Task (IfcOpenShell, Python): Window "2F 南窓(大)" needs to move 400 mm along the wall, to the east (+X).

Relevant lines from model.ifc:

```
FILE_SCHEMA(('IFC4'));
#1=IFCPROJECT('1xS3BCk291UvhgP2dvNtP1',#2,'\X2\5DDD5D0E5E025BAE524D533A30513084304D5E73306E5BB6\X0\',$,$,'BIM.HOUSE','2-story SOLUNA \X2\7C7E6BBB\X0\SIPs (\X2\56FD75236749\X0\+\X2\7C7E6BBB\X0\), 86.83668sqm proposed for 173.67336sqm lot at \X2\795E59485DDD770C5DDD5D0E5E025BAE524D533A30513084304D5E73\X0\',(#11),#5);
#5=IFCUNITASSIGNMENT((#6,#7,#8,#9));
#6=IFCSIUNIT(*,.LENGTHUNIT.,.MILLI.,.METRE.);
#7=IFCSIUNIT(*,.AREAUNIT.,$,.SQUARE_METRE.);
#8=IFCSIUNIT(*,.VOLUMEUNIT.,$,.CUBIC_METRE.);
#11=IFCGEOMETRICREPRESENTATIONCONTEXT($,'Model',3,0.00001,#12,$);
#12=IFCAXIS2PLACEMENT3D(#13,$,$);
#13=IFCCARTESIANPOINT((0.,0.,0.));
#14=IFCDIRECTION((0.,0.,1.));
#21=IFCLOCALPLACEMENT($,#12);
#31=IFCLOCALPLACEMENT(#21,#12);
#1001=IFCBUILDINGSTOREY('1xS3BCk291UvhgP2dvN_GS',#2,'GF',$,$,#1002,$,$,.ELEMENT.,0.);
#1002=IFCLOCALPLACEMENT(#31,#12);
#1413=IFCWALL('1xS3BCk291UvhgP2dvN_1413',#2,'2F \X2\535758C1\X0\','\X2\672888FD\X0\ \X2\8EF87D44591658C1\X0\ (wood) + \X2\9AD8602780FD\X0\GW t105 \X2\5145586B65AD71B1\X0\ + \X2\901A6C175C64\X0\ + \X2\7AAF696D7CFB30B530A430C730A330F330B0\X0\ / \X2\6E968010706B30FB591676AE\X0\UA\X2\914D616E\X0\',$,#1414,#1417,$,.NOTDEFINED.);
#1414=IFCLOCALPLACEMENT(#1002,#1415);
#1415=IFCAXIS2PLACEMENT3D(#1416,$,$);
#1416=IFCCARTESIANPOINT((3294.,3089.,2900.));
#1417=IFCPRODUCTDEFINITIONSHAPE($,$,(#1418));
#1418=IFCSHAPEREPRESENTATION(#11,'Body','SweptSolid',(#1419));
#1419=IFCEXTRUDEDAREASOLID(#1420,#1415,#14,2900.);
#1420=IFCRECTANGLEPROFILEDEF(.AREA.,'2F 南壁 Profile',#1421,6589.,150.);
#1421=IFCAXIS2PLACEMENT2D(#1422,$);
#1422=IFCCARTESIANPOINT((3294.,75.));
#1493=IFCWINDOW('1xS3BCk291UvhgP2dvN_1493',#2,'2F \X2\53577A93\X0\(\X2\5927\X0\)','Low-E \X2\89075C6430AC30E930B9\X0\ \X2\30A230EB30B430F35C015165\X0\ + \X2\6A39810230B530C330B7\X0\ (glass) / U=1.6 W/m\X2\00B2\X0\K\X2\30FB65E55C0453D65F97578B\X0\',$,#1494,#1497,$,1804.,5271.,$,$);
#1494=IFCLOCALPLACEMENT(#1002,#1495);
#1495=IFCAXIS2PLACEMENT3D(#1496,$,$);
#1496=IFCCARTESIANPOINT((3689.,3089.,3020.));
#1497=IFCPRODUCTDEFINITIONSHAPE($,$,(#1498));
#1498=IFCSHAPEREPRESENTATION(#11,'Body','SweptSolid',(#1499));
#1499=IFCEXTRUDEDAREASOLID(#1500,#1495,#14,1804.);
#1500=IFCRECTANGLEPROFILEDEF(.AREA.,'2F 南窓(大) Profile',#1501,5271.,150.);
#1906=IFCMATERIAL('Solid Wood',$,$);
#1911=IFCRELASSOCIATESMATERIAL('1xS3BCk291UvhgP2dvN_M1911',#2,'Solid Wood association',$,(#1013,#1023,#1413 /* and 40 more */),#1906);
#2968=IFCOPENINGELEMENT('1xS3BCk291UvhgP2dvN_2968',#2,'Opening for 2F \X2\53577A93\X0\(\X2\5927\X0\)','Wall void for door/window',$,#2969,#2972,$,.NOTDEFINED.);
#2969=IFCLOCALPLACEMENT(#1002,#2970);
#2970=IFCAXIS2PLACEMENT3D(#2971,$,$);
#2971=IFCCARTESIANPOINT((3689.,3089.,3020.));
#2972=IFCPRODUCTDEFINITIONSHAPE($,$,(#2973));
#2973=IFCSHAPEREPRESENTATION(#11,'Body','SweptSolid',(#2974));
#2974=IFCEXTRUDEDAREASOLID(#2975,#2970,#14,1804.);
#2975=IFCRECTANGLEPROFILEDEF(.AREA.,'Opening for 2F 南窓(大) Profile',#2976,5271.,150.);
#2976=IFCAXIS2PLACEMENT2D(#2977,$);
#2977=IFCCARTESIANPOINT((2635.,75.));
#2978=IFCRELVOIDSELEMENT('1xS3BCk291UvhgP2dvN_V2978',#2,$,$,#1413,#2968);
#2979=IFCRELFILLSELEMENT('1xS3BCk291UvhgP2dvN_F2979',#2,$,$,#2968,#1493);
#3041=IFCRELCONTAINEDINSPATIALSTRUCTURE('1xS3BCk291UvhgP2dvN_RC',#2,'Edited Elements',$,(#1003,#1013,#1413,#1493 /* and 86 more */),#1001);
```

```python
import ifcopenshell
import ifcopenshell.api.geometry
import ifcopenshell.util.placement
import ifcopenshell.util.unit

model = ifcopenshell.open("model.ifc")
unit_scale = ifcopenshell.util.unit.calculate_unit_scale(model)

window = model.by_guid("1xS3BCk291UvhgP2dvN_1493")
opening = window.FillsVoids[0].RelatingOpeningElement
wall = opening.VoidsElements[0].RelatingBuildingElement

wall_matrix = ifcopenshell.util.placement.get_local_placement(wall.ObjectPlacement)
shift = wall_matrix[:3, 0] * 0.4 / unit_scale
before = ifcopenshell.util.placement.get_local_placement(window.ObjectPlacement)[:3, 3].copy()

# The window is not placed relative to its opening, so move both.
for product in (opening, window):
    matrix = ifcopenshell.util.placement.get_local_placement(product.ObjectPlacement)
    matrix[:3, 3] += shift
    ifcopenshell.api.geometry.edit_object_placement(model, product=product, matrix=matrix, is_si=False)

after = ifcopenshell.util.placement.get_local_placement(window.ObjectPlacement)[:3, 3]
print("window moved by", (after - before).round(3) + 0.0)

model.write("model_rev.ifc")
```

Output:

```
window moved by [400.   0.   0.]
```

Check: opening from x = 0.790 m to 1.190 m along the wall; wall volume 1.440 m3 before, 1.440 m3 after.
